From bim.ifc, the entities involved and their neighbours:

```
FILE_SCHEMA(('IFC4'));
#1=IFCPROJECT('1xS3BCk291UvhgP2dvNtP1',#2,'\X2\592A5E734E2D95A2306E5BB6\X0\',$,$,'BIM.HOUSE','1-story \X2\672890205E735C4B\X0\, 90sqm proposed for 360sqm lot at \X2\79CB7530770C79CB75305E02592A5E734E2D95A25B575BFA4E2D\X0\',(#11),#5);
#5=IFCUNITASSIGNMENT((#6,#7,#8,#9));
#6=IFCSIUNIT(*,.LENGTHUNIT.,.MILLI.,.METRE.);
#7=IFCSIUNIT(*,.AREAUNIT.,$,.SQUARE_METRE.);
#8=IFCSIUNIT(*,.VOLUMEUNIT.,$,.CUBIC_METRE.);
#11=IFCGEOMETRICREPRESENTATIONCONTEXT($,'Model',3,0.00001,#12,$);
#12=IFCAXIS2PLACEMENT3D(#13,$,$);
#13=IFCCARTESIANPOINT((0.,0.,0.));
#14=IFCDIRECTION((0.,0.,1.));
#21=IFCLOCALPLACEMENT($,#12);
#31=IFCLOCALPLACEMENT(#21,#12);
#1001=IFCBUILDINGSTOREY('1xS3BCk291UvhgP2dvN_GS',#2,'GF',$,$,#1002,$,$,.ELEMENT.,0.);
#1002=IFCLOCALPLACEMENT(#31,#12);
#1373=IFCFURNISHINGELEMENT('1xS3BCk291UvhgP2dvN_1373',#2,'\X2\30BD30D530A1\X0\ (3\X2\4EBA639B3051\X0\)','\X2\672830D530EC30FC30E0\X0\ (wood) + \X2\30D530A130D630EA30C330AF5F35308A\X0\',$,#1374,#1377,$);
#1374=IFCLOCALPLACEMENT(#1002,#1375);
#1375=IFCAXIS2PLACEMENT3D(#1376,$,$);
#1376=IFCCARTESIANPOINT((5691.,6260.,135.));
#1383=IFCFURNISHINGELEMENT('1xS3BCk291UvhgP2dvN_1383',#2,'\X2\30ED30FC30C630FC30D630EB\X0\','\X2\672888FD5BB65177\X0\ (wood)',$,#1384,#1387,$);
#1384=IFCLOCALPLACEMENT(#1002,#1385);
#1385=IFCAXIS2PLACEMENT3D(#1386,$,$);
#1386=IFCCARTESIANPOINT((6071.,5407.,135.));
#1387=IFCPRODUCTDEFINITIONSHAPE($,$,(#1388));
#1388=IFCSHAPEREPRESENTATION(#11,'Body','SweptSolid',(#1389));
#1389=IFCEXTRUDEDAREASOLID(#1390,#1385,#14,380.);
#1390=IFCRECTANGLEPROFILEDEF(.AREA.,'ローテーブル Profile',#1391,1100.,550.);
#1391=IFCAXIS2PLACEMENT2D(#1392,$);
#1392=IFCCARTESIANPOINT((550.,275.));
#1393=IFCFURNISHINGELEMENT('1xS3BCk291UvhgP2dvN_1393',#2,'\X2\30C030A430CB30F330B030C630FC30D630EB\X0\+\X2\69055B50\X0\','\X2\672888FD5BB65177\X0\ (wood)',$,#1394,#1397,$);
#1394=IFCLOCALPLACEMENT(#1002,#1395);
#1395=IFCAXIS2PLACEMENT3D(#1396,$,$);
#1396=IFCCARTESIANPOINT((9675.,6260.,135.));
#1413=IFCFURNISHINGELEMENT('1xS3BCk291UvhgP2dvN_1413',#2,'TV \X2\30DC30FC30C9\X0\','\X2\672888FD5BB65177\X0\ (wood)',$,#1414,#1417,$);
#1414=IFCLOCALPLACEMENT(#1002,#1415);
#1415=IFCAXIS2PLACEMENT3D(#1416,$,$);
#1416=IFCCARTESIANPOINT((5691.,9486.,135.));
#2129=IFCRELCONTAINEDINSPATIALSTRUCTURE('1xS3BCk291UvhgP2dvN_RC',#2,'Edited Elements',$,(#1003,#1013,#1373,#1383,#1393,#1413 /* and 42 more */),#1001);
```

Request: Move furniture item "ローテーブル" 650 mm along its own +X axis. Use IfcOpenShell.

```python
import ifcopenshell
import ifcopenshell.api.geometry
import ifcopenshell.util.placement
import ifcopenshell.util.unit

model = ifcopenshell.open("bim.ifc")
unit_scale = ifcopenshell.util.unit.calculate_unit_scale(model)

item = model.by_guid("1xS3BCk291UvhgP2dvN_1383")
matrix = ifcopenshell.util.placement.get_local_placement(item.ObjectPlacement)
matrix[:3, 3] += matrix[:3, 0] * 0.65 / unit_scale
ifcopenshell.api.geometry.edit_object_placement(model, product=item, matrix=matrix, is_si=False)

print(ifcopenshell.util.placement.get_local_placement(item.ObjectPlacement).round(3) + 0.0)

model.write("bim_v2.ifc")
```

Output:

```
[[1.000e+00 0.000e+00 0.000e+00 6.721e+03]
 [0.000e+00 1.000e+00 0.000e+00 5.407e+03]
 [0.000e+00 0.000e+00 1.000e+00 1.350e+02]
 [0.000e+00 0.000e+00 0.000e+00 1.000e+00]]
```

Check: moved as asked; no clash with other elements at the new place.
